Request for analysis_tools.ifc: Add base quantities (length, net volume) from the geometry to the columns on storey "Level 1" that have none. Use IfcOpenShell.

First a look at what the model holds.

```python
import ifcopenshell
import ifcopenshell.util.element
import ifcopenshell.util.unit

model = ifcopenshell.open("analysis_tools.ifc")
print(model.schema)
for unit_type in ("LENGTHUNIT", "AREAUNIT", "VOLUMEUNIT"):
    print(unit_type, ifcopenshell.util.unit.calculate_unit_scale(model, unit_type))
storey = next(s for s in model.by_type("IfcBuildingStorey") if s.Name == "Level 1")
columns = [e for e in ifcopenshell.util.element.get_decomposition(storey) if e.is_a("IfcColumn")]
for e in sorted(columns, key=lambda e: e.id()):
    print(e.id(), e.is_a(), e.Name, list(ifcopenshell.util.element.get_psets(e, qtos_only=True)), sep=" | ")
```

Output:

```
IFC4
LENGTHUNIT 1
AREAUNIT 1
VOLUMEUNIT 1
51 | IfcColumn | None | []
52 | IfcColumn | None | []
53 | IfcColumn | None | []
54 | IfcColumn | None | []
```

```python
import ifcopenshell
import ifcopenshell.api.pset
import ifcopenshell.geom
import ifcopenshell.util.element
import ifcopenshell.util.shape
import ifcopenshell.util.unit

model = ifcopenshell.open("analysis_tools.ifc")
unit_scale = ifcopenshell.util.unit.calculate_unit_scale(model)
volume_scale = ifcopenshell.util.unit.calculate_unit_scale(model, "VOLUMEUNIT")
settings = ifcopenshell.geom.settings()

storey = next(s for s in model.by_type("IfcBuildingStorey") if s.Name == "Level 1")
columns = [e for e in ifcopenshell.util.element.get_decomposition(storey) if e.is_a("IfcColumn")]

for e in sorted(columns, key=lambda e: e.id()):
    if ifcopenshell.util.element.get_psets(e, qtos_only=True, should_inherit=False):
        continue
    # Geometry comes back in metres, in the element's own axes.
    shape = ifcopenshell.geom.create_shape(settings, e)
    values = {
        "Length": ifcopenshell.util.shape.get_z(shape.geometry) / unit_scale,
        "NetVolume": ifcopenshell.util.shape.get_volume(shape.geometry) / volume_scale,
    }
    qto = ifcopenshell.api.pset.add_qto(model, product=e, name="Qto_ColumnBaseQuantities")
    ifcopenshell.api.pset.edit_qto(model, qto=qto, properties=values)
    print(e.id(), {k: round(v, 3) for k, v in values.items()})

model.write("analysis_tools_rev.ifc")
```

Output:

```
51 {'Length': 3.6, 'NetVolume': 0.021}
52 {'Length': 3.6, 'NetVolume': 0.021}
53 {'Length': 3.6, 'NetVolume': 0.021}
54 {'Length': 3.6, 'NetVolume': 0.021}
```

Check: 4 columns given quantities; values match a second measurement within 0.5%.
